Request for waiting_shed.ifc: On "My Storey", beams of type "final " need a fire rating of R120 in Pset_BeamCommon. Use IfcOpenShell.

First a look at what the model holds.

```python
import ifcopenshell
import ifcopenshell.util.element

model = ifcopenshell.open("waiting_shed.ifc")
print(model.schema)
storey = next(s for s in model.by_type("IfcBuildingStorey") if s.Name == "My Storey")
beams = [e for e in ifcopenshell.util.element.get_decomposition(storey) if e.is_a("IfcBeam")]
seen = {}
for e in beams:
    element_type = ifcopenshell.util.element.get_type(e)
    key = (element_type.Name if element_type != e and element_type else None, ifcopenshell.util.element.get_pset(e, "Pset_BeamCommon", "FireRating"))
    seen[key] = seen.get(key, 0) + 1
for (name, value), count in sorted(seen.items(), key=str):
    print(count, "x", name, "|", value)
```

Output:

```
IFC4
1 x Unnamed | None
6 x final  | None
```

```python
import ifcopenshell
import ifcopenshell.api.pset
import ifcopenshell.util.element

model = ifcopenshell.open("waiting_shed.ifc")

storey = next(s for s in model.by_type("IfcBuildingStorey") if s.Name == "My Storey")
beams = [e for e in ifcopenshell.util.element.get_decomposition(storey) if e.is_a("IfcBeam")]

count = 0
for e in beams:
    element_type = ifcopenshell.util.element.get_type(e)
    if element_type in (None, e) or element_type.Name != "final ":
        continue
    # add_pset returns the element's existing set when there is one.
    pset = ifcopenshell.api.pset.add_pset(model, product=e, name="Pset_BeamCommon")
    ifcopenshell.api.pset.edit_pset(model, pset=pset, properties={"FireRating": "R120"})
    count += 1

print(count, "beams updated")

model.write("waiting_shed_edited.ifc")
```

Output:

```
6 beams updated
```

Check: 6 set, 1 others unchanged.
